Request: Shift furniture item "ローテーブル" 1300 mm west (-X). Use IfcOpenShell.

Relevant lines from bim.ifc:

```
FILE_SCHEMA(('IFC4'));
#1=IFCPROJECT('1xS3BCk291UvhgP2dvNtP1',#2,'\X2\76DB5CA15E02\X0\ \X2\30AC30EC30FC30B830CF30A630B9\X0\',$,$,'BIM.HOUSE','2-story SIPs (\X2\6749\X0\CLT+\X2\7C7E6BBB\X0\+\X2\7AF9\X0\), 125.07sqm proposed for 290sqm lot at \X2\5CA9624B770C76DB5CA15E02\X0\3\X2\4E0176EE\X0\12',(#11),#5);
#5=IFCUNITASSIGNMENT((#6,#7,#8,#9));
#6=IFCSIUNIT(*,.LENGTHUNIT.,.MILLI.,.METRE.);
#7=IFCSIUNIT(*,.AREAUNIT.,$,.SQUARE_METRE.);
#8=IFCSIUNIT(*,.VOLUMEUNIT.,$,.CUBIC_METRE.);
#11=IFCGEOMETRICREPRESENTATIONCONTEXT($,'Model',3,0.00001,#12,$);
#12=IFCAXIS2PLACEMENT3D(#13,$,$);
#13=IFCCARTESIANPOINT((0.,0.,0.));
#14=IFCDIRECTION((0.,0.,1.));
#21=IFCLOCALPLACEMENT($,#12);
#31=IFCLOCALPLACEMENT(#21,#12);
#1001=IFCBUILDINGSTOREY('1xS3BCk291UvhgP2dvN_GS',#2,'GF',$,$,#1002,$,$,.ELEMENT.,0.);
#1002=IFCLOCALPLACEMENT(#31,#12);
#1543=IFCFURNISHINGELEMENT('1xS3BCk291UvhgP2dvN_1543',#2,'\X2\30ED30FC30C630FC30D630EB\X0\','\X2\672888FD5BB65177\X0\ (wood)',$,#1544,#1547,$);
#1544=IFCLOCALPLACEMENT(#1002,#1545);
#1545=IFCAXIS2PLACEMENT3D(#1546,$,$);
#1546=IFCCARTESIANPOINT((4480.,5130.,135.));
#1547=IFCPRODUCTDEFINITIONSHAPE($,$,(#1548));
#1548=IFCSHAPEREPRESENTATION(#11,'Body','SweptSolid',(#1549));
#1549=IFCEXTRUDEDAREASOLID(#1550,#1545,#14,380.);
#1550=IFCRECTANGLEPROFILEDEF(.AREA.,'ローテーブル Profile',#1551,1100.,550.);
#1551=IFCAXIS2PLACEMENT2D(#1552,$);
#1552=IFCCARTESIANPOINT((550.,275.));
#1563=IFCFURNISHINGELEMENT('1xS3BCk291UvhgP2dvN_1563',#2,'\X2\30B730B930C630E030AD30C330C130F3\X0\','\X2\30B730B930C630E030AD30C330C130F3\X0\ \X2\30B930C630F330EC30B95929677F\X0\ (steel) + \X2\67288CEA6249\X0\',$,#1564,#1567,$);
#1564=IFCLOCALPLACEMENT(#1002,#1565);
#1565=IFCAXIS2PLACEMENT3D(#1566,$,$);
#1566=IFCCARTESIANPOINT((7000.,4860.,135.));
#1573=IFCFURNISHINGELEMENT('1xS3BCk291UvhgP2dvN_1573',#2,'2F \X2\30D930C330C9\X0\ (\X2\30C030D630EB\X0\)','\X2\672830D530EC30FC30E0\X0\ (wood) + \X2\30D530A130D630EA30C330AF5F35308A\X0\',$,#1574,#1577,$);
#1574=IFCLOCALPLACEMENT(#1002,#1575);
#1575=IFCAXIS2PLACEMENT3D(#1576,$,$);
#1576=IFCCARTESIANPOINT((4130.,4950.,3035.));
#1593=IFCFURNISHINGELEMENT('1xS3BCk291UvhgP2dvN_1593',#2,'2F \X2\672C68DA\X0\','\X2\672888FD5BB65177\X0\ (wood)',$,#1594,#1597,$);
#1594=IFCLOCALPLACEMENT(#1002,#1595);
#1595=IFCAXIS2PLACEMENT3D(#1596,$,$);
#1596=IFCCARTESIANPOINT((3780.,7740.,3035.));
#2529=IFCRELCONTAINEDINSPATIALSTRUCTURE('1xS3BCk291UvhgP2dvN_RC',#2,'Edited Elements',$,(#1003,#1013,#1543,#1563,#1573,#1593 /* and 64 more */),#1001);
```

```python
import ifcopenshell
import ifcopenshell.api.geometry
import ifcopenshell.util.placement
import ifcopenshell.util.unit

model = ifcopenshell.open("bim.ifc")
unit_scale = ifcopenshell.util.unit.calculate_unit_scale(model)

item = model.by_id(1543)
matrix = ifcopenshell.util.placement.get_local_placement(item.ObjectPlacement)
matrix[0, 3] -= 1.3 / unit_scale
ifcopenshell.api.geometry.edit_object_placement(model, product=item, matrix=matrix, is_si=False)

print(ifcopenshell.util.placement.get_local_placement(item.ObjectPlacement).round(3) + 0.0)

model.write("bim_v2.ifc")
```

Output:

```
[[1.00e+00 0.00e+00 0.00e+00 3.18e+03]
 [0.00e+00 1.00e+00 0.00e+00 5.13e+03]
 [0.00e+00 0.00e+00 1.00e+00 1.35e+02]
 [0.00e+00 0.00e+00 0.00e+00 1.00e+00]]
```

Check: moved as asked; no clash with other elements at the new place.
